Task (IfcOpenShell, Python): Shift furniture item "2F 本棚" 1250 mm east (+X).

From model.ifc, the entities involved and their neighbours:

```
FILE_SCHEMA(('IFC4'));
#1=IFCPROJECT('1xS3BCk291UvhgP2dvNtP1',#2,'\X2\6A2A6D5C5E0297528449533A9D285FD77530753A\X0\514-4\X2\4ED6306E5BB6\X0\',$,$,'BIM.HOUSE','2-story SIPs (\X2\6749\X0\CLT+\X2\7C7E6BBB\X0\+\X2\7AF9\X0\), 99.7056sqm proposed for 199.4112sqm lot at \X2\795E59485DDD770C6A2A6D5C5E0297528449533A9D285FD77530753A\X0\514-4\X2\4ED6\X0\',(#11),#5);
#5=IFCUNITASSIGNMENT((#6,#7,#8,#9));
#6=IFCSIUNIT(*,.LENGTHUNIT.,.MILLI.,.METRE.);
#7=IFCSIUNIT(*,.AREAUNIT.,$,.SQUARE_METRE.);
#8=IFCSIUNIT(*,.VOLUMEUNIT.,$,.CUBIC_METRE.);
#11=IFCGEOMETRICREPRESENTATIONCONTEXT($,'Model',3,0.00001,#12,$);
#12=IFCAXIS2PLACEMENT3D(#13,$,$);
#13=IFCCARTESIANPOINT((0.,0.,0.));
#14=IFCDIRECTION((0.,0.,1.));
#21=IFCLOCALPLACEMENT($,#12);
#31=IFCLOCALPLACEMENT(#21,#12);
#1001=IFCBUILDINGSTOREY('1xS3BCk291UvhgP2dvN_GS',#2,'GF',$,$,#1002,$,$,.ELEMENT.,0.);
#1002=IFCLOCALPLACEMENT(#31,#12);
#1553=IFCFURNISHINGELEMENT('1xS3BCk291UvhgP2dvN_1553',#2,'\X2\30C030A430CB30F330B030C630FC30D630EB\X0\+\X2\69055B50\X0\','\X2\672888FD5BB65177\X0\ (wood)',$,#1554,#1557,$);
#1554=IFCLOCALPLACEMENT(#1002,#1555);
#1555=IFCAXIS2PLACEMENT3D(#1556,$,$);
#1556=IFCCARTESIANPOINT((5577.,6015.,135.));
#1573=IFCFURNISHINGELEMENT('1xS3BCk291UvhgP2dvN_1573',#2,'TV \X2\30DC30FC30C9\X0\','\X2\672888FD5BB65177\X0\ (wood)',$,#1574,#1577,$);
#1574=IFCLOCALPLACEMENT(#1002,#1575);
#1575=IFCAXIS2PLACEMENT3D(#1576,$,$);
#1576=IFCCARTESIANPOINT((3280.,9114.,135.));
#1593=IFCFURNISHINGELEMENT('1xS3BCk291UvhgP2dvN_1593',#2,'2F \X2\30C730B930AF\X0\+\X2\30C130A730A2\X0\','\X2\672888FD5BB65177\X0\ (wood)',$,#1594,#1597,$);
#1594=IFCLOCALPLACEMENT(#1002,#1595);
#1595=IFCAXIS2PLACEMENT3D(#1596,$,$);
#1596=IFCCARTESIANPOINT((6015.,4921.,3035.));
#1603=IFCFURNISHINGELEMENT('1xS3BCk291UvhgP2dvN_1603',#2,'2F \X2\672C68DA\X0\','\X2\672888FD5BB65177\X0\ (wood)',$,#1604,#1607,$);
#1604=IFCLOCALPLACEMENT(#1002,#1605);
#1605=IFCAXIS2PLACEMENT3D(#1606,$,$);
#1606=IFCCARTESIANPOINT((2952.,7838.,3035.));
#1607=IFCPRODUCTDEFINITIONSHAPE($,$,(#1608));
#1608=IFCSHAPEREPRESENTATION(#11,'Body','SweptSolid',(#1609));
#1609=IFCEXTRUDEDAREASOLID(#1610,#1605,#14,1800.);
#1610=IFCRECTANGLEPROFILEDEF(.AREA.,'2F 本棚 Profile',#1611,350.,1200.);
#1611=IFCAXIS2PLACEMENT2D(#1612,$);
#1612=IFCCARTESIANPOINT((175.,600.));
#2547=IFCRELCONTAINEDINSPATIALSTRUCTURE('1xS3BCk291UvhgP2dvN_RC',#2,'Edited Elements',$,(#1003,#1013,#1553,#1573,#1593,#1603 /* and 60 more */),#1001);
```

```python
import ifcopenshell
import ifcopenshell.api.geometry
import ifcopenshell.util.placement

model = ifcopenshell.open("model.ifc")

item = model.by_guid("1xS3BCk291UvhgP2dvN_1603")
matrix = ifcopenshell.util.placement.get_local_placement(item.ObjectPlacement)
matrix[0, 3] += 1250.0
ifcopenshell.api.geometry.edit_object_placement(model, product=item, matrix=matrix, is_si=False)

print(ifcopenshell.util.placement.get_local_placement(item.ObjectPlacement).round(3) + 0.0)

model.write("model_rev.ifc")
```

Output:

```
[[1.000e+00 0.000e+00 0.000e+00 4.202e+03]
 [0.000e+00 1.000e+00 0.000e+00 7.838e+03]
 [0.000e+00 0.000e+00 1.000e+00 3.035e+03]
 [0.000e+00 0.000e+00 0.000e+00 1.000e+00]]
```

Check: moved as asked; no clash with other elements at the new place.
